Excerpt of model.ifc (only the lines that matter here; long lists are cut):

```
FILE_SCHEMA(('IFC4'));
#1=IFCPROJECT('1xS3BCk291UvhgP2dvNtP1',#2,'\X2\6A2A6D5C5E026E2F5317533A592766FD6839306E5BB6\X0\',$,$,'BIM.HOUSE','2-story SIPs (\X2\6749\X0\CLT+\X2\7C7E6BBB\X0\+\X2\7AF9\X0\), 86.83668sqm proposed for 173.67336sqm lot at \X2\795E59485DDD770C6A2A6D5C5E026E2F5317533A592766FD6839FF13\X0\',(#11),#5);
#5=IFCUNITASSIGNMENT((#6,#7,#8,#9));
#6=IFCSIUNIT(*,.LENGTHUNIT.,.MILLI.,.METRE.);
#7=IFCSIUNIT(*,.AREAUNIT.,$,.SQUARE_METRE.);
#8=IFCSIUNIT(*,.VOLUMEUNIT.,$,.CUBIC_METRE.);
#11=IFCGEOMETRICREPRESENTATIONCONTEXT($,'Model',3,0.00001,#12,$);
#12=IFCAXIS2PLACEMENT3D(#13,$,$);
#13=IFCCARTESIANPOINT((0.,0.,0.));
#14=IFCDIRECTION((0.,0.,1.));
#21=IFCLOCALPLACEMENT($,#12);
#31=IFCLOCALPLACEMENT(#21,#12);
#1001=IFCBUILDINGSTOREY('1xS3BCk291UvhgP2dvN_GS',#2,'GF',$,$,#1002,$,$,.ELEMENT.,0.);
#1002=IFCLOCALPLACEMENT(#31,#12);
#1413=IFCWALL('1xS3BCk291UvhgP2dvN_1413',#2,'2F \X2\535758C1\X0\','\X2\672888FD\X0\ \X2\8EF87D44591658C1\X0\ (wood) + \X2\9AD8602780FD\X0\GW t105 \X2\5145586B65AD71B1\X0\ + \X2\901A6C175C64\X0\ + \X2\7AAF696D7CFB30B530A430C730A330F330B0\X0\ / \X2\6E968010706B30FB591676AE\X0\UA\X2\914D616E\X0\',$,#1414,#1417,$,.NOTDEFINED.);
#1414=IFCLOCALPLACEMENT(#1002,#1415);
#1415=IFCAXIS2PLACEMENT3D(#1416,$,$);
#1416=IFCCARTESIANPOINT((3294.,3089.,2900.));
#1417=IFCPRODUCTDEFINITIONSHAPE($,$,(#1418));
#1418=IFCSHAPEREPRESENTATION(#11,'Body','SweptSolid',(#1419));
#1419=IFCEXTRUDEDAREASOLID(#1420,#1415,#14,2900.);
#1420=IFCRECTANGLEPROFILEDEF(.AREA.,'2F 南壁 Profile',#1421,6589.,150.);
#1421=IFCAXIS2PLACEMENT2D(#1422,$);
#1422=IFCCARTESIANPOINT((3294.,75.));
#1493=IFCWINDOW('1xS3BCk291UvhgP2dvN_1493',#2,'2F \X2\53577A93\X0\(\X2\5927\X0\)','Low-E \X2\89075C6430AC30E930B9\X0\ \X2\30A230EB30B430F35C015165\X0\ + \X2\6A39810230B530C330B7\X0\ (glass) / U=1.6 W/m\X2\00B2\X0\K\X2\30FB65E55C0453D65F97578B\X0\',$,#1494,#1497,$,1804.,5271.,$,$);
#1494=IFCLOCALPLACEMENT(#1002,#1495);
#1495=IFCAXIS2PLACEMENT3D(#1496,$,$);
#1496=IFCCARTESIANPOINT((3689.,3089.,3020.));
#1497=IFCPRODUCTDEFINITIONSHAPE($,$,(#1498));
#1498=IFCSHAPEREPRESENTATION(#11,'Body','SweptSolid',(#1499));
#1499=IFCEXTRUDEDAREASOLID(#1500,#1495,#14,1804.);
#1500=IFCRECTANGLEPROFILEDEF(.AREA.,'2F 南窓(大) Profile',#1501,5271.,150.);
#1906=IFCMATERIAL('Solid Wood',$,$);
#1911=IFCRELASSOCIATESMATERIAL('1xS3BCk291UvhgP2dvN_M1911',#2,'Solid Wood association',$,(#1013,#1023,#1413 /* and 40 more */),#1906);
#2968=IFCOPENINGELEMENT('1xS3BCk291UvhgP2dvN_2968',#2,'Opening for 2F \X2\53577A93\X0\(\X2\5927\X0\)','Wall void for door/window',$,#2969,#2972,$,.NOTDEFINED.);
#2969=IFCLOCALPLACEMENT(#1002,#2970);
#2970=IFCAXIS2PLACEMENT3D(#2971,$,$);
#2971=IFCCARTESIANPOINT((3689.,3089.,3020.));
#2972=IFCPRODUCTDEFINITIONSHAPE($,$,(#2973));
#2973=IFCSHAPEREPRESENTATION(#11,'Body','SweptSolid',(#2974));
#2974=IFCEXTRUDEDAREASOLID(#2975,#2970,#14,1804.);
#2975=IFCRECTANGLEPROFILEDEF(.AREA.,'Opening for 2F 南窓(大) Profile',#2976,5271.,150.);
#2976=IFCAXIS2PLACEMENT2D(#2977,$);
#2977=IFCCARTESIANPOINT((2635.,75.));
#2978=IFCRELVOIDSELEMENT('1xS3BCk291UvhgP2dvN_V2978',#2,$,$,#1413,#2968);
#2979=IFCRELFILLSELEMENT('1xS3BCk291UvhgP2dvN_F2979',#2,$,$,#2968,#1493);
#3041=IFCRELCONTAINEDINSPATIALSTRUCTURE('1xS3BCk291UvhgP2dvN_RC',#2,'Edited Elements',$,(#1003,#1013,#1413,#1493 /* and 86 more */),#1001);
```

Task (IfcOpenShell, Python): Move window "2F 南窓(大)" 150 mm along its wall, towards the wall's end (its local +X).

```python
import ifcopenshell
import ifcopenshell.api.geometry
import ifcopenshell.util.placement
import ifcopenshell.util.unit

model = ifcopenshell.open("model.ifc")
unit_scale = ifcopenshell.util.unit.calculate_unit_scale(model)

window = model.by_guid("1xS3BCk291UvhgP2dvN_1493")
opening = window.FillsVoids[0].RelatingOpeningElement
wall = opening.VoidsElements[0].RelatingBuildingElement

wall_matrix = ifcopenshell.util.placement.get_local_placement(wall.ObjectPlacement)
shift = wall_matrix[:3, 0] * 0.15 / unit_scale
before = ifcopenshell.util.placement.get_local_placement(window.ObjectPlacement)[:3, 3].copy()

# The window is not placed relative to its opening, so move both.
for product in (opening, window):
    matrix = ifcopenshell.util.placement.get_local_placement(product.ObjectPlacement)
    matrix[:3, 3] += shift
    ifcopenshell.api.geometry.edit_object_placement(model, product=product, matrix=matrix, is_si=False)

after = ifcopenshell.util.placement.get_local_placement(window.ObjectPlacement)[:3, 3]
print("window moved by", (after - before).round(3) + 0.0)

model.write("model_edited.ifc")
```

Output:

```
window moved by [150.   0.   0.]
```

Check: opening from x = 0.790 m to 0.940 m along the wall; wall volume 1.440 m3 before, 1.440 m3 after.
